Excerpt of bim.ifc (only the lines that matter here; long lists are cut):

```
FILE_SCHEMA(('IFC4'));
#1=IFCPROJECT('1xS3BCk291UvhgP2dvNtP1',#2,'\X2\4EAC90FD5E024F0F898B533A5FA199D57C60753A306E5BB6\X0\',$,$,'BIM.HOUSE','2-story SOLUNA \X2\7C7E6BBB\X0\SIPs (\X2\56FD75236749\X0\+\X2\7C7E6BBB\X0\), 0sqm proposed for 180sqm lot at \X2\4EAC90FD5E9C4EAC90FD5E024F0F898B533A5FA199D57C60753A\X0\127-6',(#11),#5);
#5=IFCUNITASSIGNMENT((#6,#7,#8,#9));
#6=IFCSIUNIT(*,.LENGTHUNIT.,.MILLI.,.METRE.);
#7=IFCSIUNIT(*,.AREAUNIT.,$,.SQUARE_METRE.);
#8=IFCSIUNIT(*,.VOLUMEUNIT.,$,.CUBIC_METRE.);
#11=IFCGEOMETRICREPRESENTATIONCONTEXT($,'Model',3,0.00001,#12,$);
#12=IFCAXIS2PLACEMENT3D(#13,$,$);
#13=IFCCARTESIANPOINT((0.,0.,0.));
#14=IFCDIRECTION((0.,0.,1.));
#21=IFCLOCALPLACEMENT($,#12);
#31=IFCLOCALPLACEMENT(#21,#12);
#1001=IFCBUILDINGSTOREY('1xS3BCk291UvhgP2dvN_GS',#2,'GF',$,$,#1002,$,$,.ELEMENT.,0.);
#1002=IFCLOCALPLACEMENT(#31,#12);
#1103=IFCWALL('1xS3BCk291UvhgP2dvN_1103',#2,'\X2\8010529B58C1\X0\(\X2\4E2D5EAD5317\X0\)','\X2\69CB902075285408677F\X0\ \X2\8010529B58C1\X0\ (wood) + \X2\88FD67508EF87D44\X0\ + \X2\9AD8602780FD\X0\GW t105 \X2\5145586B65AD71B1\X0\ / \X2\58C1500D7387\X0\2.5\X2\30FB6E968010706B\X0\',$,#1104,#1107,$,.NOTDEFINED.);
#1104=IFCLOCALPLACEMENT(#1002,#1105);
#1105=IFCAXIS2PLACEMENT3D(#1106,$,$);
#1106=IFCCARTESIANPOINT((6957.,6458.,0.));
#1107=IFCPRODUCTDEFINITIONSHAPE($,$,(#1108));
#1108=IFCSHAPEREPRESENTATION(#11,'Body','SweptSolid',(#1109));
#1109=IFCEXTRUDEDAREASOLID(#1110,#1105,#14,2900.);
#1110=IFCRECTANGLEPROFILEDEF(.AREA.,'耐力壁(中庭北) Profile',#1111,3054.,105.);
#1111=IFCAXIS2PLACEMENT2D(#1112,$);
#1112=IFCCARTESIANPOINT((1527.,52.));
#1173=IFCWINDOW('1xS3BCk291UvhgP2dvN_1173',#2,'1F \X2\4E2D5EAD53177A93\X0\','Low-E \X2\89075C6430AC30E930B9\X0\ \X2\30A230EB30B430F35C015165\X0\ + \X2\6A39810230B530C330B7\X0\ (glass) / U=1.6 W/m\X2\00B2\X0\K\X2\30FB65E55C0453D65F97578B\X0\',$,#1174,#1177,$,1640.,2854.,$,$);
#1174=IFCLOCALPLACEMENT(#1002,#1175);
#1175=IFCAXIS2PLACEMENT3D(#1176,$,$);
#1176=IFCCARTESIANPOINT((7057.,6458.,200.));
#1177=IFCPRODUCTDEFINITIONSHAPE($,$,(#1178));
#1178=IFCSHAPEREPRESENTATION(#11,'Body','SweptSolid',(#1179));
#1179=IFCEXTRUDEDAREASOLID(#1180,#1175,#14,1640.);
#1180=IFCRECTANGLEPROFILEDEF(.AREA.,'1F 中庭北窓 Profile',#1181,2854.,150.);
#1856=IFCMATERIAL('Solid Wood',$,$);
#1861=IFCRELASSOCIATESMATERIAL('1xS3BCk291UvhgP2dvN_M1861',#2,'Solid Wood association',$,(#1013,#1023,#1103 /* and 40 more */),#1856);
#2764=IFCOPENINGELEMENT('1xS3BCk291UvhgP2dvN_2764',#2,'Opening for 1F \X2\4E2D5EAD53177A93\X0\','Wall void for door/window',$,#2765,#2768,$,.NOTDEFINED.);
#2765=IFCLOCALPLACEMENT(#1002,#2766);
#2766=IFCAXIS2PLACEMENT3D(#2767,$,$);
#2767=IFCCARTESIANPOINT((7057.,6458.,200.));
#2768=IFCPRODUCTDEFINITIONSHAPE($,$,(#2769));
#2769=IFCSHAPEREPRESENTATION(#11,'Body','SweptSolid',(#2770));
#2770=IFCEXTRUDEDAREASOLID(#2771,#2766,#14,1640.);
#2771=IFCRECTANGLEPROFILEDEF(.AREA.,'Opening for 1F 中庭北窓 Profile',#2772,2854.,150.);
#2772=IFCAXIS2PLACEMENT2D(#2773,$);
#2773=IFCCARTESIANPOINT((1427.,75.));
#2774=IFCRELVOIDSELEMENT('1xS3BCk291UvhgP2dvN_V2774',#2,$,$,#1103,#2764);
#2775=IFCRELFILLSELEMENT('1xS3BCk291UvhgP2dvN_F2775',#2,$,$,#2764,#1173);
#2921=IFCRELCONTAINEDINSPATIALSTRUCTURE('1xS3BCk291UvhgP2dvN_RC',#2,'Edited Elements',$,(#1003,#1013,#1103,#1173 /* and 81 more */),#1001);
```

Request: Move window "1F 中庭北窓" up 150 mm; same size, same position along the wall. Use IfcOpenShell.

```python
import numpy as np
import ifcopenshell
import ifcopenshell.api.geometry
import ifcopenshell.util.placement
import ifcopenshell.util.unit

model = ifcopenshell.open("bim.ifc")
unit_scale = ifcopenshell.util.unit.calculate_unit_scale(model)

window = model.by_guid("1xS3BCk291UvhgP2dvN_1173")
opening = window.FillsVoids[0].RelatingOpeningElement
dz = 0.15 / unit_scale

shift = np.array([0.0, 0.0, dz])
# The window is not placed relative to its opening, so move both.
for product in (opening, window):
    matrix = ifcopenshell.util.placement.get_local_placement(product.ObjectPlacement)
    matrix[:3, 3] += shift
    ifcopenshell.api.geometry.edit_object_placement(model, product=product, matrix=matrix, is_si=False)

print(f"moved by {dz * unit_scale:+.3f} m")

model.write("bim-out.ifc")
```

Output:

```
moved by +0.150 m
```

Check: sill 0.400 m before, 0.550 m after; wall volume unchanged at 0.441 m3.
